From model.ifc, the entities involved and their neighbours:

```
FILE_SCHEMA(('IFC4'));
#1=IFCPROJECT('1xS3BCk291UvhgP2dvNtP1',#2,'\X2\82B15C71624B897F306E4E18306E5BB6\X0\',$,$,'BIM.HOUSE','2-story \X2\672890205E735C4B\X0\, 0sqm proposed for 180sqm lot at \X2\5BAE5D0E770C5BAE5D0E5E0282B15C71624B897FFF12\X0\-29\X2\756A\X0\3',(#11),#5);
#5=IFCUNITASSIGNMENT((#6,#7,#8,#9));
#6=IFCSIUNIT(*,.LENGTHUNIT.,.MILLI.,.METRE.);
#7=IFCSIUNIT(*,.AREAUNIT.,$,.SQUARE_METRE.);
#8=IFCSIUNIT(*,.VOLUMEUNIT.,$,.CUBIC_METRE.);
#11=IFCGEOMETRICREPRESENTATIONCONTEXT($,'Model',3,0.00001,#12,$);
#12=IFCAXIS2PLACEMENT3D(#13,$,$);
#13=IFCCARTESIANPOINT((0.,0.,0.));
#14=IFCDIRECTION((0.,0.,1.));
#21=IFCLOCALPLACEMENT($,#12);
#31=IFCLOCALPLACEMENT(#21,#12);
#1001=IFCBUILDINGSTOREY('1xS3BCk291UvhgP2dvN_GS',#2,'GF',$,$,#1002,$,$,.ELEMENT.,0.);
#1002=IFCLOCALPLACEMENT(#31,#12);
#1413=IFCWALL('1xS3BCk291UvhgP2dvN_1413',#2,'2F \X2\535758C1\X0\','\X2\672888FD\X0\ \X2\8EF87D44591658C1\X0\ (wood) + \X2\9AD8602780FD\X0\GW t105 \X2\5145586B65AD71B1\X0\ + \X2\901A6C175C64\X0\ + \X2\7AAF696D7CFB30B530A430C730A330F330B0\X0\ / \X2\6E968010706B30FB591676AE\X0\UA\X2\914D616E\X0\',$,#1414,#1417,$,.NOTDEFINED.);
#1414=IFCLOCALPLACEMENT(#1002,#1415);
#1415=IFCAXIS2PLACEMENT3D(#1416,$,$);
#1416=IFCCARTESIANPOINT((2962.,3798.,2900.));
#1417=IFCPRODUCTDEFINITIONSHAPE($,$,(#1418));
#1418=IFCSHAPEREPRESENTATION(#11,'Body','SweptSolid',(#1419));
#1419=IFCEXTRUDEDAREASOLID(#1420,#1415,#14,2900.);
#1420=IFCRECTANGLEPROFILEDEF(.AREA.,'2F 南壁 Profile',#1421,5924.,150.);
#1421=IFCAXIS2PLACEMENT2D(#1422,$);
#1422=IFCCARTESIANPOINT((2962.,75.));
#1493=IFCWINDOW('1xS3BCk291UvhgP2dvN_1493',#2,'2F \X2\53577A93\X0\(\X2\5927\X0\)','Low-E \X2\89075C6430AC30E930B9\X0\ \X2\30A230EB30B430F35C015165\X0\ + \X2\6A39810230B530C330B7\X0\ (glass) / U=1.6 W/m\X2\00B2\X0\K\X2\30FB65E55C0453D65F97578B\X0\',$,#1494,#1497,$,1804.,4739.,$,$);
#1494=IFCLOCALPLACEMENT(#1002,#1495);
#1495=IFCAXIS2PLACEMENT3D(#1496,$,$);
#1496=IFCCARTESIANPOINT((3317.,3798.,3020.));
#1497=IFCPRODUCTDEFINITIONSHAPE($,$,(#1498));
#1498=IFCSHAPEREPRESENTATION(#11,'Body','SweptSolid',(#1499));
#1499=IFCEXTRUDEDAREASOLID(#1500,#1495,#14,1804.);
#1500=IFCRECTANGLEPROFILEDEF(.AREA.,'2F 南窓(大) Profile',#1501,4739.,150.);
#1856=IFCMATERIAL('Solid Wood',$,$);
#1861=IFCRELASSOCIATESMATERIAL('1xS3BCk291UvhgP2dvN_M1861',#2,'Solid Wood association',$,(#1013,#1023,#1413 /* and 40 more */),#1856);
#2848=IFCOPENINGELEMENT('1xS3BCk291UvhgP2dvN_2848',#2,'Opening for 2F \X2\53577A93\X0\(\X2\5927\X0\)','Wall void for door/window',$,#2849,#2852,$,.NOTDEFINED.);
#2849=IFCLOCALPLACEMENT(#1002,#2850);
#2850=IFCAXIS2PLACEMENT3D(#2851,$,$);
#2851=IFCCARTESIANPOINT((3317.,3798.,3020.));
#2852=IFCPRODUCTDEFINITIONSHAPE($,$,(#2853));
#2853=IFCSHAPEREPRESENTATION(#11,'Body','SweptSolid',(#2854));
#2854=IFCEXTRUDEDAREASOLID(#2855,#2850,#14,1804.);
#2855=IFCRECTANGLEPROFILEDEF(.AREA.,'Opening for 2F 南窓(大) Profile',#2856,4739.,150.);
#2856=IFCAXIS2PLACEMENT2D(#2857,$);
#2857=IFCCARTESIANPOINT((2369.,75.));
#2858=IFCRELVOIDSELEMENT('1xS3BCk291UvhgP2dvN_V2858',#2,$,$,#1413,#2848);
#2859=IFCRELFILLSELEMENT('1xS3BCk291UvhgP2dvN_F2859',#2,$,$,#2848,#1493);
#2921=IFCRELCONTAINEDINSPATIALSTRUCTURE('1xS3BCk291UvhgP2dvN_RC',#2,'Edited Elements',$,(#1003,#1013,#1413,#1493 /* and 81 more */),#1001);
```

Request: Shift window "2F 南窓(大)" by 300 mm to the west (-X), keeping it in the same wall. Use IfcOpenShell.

```python
import ifcopenshell
import ifcopenshell.api.geometry
import ifcopenshell.util.placement
import ifcopenshell.util.unit

model = ifcopenshell.open("model.ifc")
unit_scale = ifcopenshell.util.unit.calculate_unit_scale(model)

window = model.by_id(1493)
opening = window.FillsVoids[0].RelatingOpeningElement
wall = opening.VoidsElements[0].RelatingBuildingElement

wall_matrix = ifcopenshell.util.placement.get_local_placement(wall.ObjectPlacement)
shift = wall_matrix[:3, 0] * -0.3 / unit_scale
before = ifcopenshell.util.placement.get_local_placement(window.ObjectPlacement)[:3, 3].copy()

# The window is not placed relative to its opening, so move both.
for product in (opening, window):
    matrix = ifcopenshell.util.placement.get_local_placement(product.ObjectPlacement)
    matrix[:3, 3] += shift
    ifcopenshell.api.geometry.edit_object_placement(model, product=product, matrix=matrix, is_si=False)

after = ifcopenshell.util.placement.get_local_placement(window.ObjectPlacement)[:3, 3]
print("window moved by", (after - before).round(3) + 0.0)

model.write("model_rev.ifc")
```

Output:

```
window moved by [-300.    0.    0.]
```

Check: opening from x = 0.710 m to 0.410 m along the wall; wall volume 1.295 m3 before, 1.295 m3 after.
